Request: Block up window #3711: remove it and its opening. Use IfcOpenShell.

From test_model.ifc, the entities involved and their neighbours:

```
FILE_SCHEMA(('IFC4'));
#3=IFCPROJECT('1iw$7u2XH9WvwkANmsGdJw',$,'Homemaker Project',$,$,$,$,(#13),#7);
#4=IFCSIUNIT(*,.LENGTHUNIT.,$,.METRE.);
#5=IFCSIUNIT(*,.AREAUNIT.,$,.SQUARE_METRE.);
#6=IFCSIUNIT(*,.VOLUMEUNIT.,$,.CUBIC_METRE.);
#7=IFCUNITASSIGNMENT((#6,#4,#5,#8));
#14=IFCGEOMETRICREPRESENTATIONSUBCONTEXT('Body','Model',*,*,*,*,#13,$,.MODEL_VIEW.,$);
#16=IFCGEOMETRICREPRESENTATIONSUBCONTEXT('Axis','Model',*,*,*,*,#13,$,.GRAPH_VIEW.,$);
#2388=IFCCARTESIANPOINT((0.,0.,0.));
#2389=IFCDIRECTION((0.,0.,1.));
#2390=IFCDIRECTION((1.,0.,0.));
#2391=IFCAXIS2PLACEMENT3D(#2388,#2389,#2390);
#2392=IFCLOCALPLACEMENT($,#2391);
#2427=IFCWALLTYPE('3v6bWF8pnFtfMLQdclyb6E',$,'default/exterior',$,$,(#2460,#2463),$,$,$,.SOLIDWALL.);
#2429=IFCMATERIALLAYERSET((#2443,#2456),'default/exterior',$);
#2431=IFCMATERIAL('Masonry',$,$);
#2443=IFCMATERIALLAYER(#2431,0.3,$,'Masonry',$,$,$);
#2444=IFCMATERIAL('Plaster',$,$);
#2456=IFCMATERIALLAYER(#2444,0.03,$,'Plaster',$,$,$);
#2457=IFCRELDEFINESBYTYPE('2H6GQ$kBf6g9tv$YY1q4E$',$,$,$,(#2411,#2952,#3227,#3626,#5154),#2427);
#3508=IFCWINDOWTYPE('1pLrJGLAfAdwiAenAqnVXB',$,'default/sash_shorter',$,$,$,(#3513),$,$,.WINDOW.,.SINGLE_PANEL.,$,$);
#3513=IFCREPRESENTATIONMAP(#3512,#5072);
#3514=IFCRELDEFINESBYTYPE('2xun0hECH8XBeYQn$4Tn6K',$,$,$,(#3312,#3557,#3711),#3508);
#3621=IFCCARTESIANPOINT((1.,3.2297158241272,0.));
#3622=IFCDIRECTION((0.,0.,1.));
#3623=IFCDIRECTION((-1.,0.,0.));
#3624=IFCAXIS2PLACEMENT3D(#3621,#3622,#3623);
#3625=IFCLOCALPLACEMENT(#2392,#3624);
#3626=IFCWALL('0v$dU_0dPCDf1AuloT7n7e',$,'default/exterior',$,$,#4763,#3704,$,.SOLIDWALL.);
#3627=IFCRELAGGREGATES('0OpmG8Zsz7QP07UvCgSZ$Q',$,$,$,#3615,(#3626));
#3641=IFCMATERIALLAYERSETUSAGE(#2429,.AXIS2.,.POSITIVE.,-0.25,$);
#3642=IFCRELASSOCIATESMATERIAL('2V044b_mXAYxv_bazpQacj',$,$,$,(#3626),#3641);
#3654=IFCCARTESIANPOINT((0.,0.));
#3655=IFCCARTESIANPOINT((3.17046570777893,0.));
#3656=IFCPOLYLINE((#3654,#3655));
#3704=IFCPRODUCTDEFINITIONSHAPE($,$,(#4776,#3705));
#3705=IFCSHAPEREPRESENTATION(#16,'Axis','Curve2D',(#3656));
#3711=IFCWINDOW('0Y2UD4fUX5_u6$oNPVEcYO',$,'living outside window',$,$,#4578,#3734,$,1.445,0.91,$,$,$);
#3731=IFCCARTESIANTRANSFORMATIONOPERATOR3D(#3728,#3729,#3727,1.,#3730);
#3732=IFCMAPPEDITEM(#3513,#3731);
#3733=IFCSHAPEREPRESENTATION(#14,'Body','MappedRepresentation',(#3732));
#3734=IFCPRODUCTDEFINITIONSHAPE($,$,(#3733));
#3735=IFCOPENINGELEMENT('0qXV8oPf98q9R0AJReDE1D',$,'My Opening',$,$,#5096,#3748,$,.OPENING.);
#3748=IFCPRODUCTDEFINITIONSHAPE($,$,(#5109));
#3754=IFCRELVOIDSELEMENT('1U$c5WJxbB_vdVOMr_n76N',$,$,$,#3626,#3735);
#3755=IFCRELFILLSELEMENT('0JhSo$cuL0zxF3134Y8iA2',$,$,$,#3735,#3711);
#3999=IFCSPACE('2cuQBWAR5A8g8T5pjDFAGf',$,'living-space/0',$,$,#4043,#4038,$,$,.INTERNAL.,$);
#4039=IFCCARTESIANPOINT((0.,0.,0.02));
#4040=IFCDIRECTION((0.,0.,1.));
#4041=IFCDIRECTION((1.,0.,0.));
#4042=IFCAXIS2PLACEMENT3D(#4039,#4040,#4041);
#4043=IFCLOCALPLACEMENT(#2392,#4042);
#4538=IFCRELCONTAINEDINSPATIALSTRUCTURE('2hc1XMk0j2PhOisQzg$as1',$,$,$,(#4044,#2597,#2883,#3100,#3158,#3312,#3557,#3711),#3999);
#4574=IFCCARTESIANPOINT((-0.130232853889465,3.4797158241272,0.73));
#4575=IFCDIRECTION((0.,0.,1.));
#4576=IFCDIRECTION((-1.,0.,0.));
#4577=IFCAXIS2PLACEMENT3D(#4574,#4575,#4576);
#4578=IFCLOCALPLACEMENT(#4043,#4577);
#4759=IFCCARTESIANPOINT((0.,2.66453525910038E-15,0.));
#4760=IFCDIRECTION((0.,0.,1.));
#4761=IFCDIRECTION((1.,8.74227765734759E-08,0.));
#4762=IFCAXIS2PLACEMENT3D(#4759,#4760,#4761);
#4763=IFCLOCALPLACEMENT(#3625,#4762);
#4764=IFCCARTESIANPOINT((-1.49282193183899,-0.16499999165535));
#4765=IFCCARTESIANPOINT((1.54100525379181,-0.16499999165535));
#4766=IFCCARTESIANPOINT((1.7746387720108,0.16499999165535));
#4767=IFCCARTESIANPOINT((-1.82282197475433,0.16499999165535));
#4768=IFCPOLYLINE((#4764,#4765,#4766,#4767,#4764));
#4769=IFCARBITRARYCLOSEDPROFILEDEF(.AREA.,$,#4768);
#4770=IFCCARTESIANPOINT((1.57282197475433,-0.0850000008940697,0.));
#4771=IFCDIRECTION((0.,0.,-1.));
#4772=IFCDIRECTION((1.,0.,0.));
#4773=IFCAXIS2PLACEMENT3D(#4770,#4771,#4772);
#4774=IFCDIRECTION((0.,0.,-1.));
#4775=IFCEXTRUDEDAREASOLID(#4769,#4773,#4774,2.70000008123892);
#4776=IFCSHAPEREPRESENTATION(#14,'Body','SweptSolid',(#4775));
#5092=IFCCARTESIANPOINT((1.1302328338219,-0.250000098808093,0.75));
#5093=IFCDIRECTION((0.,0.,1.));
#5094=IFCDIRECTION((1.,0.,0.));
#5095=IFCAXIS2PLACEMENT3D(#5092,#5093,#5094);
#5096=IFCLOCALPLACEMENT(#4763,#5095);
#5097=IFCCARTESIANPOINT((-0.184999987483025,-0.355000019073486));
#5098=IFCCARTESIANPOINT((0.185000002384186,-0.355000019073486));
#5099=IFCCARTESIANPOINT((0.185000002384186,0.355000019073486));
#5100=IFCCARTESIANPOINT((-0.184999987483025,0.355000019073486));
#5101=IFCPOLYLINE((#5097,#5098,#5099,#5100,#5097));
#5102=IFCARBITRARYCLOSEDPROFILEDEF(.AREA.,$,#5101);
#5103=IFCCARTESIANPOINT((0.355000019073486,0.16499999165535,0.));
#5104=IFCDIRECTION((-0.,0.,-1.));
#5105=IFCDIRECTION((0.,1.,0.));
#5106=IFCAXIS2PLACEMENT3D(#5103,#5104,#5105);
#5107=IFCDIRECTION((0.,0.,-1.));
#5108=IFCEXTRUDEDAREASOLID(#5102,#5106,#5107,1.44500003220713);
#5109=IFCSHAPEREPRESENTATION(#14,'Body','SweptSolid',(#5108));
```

```python
import ifcopenshell
import ifcopenshell.api.feature
import ifcopenshell.api.root
import ifcopenshell.geom
import ifcopenshell.util.shape

model = ifcopenshell.open("test_model.ifc")
settings = ifcopenshell.geom.settings()


def volume(element):
    """Net volume in cubic metres, openings subtracted."""
    shape = ifcopenshell.geom.create_shape(settings, element)
    return ifcopenshell.util.shape.get_volume(shape.geometry)


window = model.by_guid("0Y2UD4fUX5_u6$oNPVEcYO")
opening = window.FillsVoids[0].RelatingOpeningElement
wall = opening.VoidsElements[0].RelatingBuildingElement
before = volume(wall)

ifcopenshell.api.root.remove_product(model, product=window)
ifcopenshell.api.feature.remove_feature(model, feature=opening)

after = volume(wall)

print(f"wall volume {before:.3f} -> {after:.3f} m3")

model.write("test_model-out.ifc")
```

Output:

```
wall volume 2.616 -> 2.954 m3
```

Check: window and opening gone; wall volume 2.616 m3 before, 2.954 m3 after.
